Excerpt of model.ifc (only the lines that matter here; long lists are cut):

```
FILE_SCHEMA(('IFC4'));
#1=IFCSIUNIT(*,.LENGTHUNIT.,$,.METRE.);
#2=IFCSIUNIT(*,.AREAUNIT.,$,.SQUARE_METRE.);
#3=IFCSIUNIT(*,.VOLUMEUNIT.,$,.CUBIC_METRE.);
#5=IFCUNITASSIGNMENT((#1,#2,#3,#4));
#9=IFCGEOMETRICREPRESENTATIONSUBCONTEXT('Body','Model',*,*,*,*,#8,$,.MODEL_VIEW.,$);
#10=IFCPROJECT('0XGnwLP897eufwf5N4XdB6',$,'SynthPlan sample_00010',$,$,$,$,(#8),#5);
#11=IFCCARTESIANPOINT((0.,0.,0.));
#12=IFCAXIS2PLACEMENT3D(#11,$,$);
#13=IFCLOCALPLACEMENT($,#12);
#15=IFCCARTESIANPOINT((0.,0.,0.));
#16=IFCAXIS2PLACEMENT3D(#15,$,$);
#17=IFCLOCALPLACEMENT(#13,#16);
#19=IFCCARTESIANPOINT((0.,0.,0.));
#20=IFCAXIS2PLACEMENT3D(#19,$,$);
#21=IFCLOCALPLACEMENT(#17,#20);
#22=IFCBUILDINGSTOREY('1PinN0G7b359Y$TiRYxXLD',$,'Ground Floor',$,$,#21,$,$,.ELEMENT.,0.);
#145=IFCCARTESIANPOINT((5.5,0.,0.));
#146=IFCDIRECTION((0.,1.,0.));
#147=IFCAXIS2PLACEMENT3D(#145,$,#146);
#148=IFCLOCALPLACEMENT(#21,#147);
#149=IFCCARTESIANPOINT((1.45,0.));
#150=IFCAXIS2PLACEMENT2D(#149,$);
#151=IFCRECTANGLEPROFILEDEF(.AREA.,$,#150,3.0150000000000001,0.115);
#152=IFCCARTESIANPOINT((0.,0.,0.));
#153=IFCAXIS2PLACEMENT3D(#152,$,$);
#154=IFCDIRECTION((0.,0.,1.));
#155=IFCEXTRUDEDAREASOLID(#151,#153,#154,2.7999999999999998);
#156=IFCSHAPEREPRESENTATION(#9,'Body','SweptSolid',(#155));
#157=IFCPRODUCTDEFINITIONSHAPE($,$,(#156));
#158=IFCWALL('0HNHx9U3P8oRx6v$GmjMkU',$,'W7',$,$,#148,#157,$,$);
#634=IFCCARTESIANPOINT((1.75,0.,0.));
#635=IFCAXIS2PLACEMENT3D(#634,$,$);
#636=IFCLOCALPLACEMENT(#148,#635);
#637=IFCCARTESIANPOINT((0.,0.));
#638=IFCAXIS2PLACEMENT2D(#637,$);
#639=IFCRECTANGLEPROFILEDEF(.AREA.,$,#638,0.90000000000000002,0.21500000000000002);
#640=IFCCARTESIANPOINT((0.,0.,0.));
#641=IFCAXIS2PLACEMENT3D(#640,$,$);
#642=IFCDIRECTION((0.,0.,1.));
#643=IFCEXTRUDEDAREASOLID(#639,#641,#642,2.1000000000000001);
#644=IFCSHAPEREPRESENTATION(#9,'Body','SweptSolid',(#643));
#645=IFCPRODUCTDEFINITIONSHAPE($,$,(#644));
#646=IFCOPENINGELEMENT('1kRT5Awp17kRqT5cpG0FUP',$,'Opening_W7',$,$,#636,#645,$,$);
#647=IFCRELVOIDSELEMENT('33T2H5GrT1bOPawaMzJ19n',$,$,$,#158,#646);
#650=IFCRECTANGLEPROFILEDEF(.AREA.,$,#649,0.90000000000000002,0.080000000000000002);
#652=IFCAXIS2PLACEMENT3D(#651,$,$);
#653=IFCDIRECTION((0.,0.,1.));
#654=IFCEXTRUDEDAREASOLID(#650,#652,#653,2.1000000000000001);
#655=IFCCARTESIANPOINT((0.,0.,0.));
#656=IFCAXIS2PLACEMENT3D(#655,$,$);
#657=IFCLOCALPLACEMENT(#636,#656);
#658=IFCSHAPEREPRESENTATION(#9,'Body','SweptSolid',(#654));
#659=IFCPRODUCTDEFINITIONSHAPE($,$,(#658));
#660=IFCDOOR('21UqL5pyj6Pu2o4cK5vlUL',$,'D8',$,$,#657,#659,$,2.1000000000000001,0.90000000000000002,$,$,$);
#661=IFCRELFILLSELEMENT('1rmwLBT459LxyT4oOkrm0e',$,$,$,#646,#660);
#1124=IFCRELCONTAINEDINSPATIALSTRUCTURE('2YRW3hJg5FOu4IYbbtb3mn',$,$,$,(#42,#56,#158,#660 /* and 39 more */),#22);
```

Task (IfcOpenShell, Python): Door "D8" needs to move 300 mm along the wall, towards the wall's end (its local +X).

```python
import ifcopenshell
import ifcopenshell.api.geometry
import ifcopenshell.util.placement

model = ifcopenshell.open("model.ifc")

door = model.by_id(660)
opening = door.FillsVoids[0].RelatingOpeningElement
wall = opening.VoidsElements[0].RelatingBuildingElement

wall_matrix = ifcopenshell.util.placement.get_local_placement(wall.ObjectPlacement)
shift = wall_matrix[:3, 0] * 0.3
before = ifcopenshell.util.placement.get_local_placement(door.ObjectPlacement)[:3, 3].copy()

# The door is placed relative to its opening, so it follows when the opening moves.
matrix = ifcopenshell.util.placement.get_local_placement(opening.ObjectPlacement)
matrix[:3, 3] += shift
ifcopenshell.api.geometry.edit_object_placement(
    model, product=opening, matrix=matrix, is_si=False, should_transform_children=True
)

after = ifcopenshell.util.placement.get_local_placement(door.ObjectPlacement)[:3, 3]
print("door moved by", (after - before).round(3) + 0.0)

model.write("model_updated.ifc")
```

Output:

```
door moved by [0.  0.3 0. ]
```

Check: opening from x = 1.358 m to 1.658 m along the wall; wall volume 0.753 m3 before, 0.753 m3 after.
